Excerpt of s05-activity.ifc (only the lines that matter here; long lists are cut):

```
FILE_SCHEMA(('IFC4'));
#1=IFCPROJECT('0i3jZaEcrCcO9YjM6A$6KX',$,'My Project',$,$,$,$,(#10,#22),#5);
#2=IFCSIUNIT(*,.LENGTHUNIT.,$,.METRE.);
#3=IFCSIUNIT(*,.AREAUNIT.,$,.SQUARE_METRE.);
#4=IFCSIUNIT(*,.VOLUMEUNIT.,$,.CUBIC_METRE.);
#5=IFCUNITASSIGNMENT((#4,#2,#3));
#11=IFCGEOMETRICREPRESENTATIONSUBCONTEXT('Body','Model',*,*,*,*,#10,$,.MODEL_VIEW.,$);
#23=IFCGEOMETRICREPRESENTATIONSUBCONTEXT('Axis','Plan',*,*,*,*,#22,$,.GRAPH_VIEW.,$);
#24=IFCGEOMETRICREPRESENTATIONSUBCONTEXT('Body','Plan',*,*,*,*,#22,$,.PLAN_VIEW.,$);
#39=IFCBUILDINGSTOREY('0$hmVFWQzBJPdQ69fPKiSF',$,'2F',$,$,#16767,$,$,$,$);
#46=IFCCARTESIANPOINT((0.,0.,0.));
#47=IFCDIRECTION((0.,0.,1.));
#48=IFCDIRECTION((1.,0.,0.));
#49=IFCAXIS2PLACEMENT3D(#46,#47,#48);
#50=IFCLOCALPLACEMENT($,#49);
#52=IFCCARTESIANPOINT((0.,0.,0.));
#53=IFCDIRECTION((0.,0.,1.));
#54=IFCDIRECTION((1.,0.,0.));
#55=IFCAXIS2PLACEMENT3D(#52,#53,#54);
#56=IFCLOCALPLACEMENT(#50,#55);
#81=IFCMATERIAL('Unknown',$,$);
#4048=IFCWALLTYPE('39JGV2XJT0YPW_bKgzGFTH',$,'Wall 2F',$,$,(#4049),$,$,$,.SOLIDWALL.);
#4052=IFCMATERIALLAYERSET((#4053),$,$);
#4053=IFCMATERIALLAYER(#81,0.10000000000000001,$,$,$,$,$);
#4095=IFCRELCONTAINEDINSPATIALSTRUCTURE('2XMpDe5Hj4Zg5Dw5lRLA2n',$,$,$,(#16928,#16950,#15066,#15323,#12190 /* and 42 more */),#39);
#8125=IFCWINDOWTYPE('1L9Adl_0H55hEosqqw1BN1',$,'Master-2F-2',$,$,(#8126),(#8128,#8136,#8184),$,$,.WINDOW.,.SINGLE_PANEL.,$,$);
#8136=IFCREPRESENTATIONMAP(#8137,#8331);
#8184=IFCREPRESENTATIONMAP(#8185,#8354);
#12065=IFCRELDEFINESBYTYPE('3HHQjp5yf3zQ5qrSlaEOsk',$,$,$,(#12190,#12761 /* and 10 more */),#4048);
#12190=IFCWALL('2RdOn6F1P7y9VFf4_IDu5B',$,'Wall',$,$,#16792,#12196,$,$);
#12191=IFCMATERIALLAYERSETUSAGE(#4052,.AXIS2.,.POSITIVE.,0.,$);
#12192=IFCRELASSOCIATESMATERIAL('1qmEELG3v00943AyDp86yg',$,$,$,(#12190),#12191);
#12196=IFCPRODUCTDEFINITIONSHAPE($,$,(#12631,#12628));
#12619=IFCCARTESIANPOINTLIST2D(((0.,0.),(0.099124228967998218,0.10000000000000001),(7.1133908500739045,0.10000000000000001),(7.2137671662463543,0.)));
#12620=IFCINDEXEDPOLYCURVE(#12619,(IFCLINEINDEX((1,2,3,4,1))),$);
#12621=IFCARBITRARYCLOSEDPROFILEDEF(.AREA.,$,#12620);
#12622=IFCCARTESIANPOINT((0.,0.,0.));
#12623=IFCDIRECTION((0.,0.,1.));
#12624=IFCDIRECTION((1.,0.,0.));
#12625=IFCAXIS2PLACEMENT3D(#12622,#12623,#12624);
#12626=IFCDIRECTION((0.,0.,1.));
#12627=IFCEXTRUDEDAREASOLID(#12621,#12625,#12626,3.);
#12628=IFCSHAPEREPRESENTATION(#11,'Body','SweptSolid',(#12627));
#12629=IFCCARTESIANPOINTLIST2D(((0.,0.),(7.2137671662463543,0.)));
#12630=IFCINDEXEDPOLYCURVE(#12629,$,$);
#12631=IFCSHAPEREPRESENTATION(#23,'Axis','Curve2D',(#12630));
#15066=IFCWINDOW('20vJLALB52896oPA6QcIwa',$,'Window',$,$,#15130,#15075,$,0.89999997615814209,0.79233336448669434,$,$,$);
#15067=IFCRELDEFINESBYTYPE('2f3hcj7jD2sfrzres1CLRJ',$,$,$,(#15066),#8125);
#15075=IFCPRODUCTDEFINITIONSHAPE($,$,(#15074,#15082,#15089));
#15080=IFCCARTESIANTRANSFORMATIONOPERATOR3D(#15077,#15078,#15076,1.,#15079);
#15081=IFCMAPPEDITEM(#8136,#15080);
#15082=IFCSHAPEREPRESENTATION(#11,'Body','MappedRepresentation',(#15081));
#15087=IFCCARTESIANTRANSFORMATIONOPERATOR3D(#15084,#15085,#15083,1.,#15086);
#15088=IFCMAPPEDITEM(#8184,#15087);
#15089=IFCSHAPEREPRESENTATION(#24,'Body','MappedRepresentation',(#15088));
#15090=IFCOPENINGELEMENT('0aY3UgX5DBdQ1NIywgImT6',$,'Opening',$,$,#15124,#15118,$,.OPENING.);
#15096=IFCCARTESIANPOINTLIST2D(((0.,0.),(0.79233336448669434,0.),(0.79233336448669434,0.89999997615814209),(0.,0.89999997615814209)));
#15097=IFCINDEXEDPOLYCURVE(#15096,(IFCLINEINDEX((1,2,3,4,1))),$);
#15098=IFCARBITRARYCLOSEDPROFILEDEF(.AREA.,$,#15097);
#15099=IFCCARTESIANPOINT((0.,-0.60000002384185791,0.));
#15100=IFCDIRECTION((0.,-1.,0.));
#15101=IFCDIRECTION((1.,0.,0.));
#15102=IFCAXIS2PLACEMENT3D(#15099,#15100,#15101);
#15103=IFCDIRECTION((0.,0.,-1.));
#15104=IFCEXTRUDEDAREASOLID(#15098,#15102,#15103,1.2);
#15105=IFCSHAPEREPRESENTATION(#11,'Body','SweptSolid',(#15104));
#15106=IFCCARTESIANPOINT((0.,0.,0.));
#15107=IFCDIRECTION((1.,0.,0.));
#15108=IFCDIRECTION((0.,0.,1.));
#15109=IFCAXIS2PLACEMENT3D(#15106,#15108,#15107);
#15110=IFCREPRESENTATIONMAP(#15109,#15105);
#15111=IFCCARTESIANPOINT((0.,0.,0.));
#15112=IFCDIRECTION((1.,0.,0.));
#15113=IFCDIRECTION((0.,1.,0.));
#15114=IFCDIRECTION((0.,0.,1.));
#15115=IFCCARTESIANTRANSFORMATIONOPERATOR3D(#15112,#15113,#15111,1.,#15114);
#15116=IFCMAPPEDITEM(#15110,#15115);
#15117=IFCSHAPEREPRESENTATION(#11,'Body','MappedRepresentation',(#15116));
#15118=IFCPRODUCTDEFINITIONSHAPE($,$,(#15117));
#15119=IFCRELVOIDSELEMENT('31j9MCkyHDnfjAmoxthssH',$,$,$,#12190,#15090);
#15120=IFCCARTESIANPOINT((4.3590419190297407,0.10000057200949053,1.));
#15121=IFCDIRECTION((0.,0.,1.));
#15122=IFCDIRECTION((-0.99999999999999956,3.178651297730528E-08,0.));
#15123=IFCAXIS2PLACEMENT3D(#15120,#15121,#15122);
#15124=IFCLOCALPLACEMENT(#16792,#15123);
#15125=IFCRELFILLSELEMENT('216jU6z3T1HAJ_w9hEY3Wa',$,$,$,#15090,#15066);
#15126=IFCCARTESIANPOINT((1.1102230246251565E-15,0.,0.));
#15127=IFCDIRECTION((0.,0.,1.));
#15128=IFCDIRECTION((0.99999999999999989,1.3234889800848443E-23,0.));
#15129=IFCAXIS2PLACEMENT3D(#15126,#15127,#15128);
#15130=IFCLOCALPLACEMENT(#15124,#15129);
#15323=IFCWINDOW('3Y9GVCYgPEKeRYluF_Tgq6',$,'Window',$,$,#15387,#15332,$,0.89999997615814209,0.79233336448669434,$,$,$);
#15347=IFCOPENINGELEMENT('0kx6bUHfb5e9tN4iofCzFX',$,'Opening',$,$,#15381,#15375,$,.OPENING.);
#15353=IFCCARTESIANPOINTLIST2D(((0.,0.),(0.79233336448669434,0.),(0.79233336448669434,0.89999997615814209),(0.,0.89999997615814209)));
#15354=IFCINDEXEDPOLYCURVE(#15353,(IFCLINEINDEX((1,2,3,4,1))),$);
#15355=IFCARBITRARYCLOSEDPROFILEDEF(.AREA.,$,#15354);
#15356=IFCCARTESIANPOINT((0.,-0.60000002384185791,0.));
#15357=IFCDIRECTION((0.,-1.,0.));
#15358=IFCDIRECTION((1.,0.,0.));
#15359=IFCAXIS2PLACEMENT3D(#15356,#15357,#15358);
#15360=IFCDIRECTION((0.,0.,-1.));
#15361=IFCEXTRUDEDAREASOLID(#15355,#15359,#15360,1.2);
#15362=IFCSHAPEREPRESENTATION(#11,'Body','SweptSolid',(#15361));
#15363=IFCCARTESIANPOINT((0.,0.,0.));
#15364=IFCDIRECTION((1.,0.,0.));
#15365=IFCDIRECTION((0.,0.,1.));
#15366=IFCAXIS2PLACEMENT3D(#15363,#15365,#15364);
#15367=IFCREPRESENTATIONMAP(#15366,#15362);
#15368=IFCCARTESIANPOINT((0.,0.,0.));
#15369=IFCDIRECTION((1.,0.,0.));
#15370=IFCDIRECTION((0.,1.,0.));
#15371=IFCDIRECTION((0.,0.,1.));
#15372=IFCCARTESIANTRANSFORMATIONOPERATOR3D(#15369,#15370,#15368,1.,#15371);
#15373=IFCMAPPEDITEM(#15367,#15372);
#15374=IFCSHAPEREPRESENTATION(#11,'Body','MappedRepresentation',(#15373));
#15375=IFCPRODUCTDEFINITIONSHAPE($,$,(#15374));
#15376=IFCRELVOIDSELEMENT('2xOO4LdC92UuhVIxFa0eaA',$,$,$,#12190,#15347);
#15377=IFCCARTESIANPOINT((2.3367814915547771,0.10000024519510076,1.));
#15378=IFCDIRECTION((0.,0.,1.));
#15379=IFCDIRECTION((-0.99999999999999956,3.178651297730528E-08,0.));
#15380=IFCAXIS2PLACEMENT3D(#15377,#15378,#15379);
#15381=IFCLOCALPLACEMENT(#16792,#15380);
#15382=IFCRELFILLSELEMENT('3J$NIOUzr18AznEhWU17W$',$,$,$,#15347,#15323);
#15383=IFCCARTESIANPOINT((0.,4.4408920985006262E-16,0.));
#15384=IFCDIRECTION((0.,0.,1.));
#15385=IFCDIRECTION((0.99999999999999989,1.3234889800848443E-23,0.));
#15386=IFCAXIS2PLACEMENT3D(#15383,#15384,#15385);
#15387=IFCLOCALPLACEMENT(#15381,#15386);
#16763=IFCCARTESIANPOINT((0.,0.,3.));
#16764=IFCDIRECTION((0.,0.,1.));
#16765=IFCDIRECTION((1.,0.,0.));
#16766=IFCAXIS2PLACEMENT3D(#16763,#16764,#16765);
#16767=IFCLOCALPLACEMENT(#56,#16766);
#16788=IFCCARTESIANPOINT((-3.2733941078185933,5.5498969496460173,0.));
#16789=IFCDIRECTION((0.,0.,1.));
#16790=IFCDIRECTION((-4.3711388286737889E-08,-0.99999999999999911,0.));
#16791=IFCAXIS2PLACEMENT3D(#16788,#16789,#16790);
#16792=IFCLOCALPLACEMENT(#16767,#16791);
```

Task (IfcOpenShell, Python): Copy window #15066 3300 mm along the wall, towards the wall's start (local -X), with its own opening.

```python
import ifcopenshell
import ifcopenshell.api.feature
import ifcopenshell.api.geometry
import ifcopenshell.api.root
import ifcopenshell.geom
import ifcopenshell.util.element
import ifcopenshell.util.placement
import ifcopenshell.util.shape

model = ifcopenshell.open("s05-activity.ifc")
settings = ifcopenshell.geom.settings()


def volume(element):
    """Net volume in cubic metres, openings subtracted."""
    shape = ifcopenshell.geom.create_shape(settings, element)
    return ifcopenshell.util.shape.get_volume(shape.geometry)


window = model.by_guid("20vJLALB52896oPA6QcIwa")
opening = window.FillsVoids[0].RelatingOpeningElement
wall = opening.VoidsElements[0].RelatingBuildingElement
before = volume(wall)
shift = ifcopenshell.util.placement.get_local_placement(wall.ObjectPlacement)[:3, 0] * -3.3

# copy_class copies the void relationship, type, container and properties, but no geometry.
new_opening = ifcopenshell.api.root.copy_class(model, product=opening)
new_opening.Representation = ifcopenshell.util.element.copy_deep(
    model, opening.Representation, exclude=["IfcGeometricRepresentationContext", "IfcRepresentationMap"]
)
new_window = ifcopenshell.api.root.copy_class(model, product=window)
new_window.Representation = ifcopenshell.util.element.copy_deep(
    model, window.Representation, exclude=["IfcGeometricRepresentationContext", "IfcRepresentationMap"]
)
ifcopenshell.api.feature.add_filling(model, opening=new_opening, element=new_window)

for old, new in ((opening, new_opening), (window, new_window)):
    matrix = ifcopenshell.util.placement.get_local_placement(old.ObjectPlacement)
    matrix[:3, 3] += shift
    ifcopenshell.api.geometry.edit_object_placement(model, product=new, matrix=matrix, is_si=False)

after = volume(wall)

print(f"wall volume {before:.3f} -> {after:.3f} m3")

model.write("s05-activity_edited.ifc")
```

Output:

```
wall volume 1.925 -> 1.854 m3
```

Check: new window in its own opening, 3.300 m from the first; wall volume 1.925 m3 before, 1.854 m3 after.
